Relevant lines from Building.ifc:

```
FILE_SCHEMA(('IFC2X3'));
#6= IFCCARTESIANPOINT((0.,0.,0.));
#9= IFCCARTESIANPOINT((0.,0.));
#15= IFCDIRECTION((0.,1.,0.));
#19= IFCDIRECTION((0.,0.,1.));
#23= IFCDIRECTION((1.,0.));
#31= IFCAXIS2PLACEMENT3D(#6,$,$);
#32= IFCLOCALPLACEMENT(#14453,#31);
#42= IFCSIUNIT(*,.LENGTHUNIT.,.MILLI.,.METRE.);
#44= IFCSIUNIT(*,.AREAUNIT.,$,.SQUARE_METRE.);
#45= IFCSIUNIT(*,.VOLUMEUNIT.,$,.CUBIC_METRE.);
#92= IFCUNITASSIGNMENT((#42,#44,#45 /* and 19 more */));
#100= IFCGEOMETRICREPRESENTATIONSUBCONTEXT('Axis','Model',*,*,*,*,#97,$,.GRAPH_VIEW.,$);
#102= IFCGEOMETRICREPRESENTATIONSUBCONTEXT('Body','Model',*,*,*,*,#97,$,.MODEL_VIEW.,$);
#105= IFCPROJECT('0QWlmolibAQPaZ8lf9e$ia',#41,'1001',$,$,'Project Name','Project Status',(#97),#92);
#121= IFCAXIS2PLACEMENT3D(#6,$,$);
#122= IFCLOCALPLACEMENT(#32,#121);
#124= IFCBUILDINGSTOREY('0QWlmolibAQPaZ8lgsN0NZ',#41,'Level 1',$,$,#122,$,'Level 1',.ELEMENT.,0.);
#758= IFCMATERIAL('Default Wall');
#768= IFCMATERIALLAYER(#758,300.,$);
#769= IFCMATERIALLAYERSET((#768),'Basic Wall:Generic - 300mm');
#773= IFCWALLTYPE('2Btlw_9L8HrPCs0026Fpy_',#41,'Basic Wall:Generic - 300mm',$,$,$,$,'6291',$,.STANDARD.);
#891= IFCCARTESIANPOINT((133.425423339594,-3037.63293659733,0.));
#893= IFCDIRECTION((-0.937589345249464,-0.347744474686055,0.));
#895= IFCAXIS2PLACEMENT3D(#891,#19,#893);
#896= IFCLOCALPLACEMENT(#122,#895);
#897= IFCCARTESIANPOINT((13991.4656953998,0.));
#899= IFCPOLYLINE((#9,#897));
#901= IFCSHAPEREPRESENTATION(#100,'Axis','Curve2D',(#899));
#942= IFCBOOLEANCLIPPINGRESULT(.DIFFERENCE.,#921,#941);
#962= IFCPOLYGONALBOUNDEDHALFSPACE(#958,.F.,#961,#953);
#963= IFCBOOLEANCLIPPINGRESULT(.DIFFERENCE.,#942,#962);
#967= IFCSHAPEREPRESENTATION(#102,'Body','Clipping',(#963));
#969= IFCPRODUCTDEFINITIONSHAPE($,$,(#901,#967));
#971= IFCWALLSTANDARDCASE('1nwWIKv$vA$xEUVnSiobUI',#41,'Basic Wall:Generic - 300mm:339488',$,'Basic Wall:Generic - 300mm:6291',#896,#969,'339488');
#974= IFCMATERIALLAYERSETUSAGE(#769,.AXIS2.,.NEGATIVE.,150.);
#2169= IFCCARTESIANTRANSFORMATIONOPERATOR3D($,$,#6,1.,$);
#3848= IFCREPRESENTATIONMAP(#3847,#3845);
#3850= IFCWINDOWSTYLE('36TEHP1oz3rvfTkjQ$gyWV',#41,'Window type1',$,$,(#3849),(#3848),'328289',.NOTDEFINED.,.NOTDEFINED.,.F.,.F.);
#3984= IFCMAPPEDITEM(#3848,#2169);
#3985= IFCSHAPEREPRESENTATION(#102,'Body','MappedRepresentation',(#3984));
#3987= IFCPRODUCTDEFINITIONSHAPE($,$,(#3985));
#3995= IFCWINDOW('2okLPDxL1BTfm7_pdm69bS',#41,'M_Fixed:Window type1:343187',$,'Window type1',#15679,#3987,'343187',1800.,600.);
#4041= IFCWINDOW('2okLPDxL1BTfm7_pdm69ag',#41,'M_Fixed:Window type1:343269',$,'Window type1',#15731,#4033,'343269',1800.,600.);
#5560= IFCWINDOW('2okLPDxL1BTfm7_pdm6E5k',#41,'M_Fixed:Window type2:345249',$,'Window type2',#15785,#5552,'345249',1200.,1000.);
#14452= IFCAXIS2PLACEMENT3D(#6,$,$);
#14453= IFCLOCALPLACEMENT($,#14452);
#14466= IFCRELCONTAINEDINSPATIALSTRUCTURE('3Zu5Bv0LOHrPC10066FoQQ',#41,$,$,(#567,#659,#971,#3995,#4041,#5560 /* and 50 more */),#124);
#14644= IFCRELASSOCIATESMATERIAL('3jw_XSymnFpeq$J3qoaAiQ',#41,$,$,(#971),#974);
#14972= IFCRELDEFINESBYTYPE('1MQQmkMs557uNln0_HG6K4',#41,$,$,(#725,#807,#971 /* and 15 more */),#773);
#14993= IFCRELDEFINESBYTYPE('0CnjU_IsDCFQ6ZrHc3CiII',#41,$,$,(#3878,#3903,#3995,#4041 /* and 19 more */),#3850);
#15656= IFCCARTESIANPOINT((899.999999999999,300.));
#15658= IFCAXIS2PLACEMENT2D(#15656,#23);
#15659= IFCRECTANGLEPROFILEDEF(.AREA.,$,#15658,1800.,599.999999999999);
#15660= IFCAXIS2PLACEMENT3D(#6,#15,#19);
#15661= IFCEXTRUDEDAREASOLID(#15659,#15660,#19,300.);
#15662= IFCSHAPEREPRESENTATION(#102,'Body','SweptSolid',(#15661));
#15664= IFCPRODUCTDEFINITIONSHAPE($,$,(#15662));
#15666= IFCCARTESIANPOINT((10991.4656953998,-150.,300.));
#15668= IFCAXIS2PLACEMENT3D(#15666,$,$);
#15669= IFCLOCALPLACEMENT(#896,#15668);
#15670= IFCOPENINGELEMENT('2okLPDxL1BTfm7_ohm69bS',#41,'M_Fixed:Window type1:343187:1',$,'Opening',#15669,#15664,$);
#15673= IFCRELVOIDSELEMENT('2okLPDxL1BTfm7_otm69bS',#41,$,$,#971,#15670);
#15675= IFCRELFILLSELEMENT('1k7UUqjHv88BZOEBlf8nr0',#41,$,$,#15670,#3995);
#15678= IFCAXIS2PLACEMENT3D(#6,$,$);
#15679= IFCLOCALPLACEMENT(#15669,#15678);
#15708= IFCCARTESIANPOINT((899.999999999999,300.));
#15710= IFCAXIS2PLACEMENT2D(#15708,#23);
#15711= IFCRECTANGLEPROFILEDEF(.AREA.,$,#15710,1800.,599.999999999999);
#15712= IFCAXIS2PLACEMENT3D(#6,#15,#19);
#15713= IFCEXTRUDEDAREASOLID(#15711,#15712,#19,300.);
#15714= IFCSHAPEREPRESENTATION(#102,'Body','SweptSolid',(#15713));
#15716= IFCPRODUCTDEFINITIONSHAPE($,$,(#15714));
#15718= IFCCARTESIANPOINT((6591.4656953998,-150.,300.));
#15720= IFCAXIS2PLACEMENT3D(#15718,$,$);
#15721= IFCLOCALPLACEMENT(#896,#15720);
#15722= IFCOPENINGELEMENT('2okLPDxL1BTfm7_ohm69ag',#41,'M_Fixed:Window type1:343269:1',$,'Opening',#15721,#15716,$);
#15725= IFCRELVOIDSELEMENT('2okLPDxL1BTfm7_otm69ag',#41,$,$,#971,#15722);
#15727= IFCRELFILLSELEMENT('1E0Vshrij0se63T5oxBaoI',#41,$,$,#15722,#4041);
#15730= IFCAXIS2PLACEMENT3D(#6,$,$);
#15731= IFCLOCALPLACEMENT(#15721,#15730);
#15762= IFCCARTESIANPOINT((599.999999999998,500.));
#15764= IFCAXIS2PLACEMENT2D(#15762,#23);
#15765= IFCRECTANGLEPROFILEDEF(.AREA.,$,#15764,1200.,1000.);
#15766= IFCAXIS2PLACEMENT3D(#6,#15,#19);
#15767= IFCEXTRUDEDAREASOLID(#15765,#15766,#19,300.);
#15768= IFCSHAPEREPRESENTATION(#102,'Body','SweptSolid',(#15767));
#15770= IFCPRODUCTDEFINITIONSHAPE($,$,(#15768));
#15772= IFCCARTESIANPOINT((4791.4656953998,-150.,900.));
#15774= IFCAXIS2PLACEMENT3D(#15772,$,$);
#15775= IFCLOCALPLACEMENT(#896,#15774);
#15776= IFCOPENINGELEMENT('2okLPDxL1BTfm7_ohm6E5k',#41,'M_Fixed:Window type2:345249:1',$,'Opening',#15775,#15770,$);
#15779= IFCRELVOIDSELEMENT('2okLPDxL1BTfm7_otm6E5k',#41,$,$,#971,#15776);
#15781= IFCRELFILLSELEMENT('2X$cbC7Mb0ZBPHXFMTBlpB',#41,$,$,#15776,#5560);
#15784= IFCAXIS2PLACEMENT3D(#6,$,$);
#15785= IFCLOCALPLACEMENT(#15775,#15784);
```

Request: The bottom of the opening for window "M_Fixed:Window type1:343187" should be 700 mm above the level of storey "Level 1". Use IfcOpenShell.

```python
import numpy as np
import ifcopenshell
import ifcopenshell.api.geometry
import ifcopenshell.geom
import ifcopenshell.util.element
import ifcopenshell.util.placement
import ifcopenshell.util.shape
import ifcopenshell.util.unit

model = ifcopenshell.open("Building.ifc")
unit_scale = ifcopenshell.util.unit.calculate_unit_scale(model)

window = model.by_guid("2okLPDxL1BTfm7_pdm69bS")
opening = window.FillsVoids[0].RelatingOpeningElement
storey = ifcopenshell.util.element.get_container(window, ifc_class="IfcBuildingStorey")
level = ifcopenshell.util.placement.get_local_placement(storey.ObjectPlacement)[2, 3]

# The opening's origin need not be at the sill, so measure its lowest point.
shape = ifcopenshell.geom.create_shape(ifcopenshell.geom.settings(), opening)
bottom = ifcopenshell.util.shape.get_shape_bottom_elevation(shape, shape.geometry) / unit_scale
dz = level + 0.7 / unit_scale - bottom

shift = np.array([0.0, 0.0, dz])
# The window is placed relative to its opening, so it follows when the opening moves.
matrix = ifcopenshell.util.placement.get_local_placement(opening.ObjectPlacement)
matrix[:3, 3] += shift
ifcopenshell.api.geometry.edit_object_placement(
    model, product=opening, matrix=matrix, is_si=False, should_transform_children=True
)

print(f"moved by {dz * unit_scale:+.3f} m")

model.write("Building_v2.ifc")
```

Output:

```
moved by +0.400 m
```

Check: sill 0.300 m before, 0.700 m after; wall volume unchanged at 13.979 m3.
